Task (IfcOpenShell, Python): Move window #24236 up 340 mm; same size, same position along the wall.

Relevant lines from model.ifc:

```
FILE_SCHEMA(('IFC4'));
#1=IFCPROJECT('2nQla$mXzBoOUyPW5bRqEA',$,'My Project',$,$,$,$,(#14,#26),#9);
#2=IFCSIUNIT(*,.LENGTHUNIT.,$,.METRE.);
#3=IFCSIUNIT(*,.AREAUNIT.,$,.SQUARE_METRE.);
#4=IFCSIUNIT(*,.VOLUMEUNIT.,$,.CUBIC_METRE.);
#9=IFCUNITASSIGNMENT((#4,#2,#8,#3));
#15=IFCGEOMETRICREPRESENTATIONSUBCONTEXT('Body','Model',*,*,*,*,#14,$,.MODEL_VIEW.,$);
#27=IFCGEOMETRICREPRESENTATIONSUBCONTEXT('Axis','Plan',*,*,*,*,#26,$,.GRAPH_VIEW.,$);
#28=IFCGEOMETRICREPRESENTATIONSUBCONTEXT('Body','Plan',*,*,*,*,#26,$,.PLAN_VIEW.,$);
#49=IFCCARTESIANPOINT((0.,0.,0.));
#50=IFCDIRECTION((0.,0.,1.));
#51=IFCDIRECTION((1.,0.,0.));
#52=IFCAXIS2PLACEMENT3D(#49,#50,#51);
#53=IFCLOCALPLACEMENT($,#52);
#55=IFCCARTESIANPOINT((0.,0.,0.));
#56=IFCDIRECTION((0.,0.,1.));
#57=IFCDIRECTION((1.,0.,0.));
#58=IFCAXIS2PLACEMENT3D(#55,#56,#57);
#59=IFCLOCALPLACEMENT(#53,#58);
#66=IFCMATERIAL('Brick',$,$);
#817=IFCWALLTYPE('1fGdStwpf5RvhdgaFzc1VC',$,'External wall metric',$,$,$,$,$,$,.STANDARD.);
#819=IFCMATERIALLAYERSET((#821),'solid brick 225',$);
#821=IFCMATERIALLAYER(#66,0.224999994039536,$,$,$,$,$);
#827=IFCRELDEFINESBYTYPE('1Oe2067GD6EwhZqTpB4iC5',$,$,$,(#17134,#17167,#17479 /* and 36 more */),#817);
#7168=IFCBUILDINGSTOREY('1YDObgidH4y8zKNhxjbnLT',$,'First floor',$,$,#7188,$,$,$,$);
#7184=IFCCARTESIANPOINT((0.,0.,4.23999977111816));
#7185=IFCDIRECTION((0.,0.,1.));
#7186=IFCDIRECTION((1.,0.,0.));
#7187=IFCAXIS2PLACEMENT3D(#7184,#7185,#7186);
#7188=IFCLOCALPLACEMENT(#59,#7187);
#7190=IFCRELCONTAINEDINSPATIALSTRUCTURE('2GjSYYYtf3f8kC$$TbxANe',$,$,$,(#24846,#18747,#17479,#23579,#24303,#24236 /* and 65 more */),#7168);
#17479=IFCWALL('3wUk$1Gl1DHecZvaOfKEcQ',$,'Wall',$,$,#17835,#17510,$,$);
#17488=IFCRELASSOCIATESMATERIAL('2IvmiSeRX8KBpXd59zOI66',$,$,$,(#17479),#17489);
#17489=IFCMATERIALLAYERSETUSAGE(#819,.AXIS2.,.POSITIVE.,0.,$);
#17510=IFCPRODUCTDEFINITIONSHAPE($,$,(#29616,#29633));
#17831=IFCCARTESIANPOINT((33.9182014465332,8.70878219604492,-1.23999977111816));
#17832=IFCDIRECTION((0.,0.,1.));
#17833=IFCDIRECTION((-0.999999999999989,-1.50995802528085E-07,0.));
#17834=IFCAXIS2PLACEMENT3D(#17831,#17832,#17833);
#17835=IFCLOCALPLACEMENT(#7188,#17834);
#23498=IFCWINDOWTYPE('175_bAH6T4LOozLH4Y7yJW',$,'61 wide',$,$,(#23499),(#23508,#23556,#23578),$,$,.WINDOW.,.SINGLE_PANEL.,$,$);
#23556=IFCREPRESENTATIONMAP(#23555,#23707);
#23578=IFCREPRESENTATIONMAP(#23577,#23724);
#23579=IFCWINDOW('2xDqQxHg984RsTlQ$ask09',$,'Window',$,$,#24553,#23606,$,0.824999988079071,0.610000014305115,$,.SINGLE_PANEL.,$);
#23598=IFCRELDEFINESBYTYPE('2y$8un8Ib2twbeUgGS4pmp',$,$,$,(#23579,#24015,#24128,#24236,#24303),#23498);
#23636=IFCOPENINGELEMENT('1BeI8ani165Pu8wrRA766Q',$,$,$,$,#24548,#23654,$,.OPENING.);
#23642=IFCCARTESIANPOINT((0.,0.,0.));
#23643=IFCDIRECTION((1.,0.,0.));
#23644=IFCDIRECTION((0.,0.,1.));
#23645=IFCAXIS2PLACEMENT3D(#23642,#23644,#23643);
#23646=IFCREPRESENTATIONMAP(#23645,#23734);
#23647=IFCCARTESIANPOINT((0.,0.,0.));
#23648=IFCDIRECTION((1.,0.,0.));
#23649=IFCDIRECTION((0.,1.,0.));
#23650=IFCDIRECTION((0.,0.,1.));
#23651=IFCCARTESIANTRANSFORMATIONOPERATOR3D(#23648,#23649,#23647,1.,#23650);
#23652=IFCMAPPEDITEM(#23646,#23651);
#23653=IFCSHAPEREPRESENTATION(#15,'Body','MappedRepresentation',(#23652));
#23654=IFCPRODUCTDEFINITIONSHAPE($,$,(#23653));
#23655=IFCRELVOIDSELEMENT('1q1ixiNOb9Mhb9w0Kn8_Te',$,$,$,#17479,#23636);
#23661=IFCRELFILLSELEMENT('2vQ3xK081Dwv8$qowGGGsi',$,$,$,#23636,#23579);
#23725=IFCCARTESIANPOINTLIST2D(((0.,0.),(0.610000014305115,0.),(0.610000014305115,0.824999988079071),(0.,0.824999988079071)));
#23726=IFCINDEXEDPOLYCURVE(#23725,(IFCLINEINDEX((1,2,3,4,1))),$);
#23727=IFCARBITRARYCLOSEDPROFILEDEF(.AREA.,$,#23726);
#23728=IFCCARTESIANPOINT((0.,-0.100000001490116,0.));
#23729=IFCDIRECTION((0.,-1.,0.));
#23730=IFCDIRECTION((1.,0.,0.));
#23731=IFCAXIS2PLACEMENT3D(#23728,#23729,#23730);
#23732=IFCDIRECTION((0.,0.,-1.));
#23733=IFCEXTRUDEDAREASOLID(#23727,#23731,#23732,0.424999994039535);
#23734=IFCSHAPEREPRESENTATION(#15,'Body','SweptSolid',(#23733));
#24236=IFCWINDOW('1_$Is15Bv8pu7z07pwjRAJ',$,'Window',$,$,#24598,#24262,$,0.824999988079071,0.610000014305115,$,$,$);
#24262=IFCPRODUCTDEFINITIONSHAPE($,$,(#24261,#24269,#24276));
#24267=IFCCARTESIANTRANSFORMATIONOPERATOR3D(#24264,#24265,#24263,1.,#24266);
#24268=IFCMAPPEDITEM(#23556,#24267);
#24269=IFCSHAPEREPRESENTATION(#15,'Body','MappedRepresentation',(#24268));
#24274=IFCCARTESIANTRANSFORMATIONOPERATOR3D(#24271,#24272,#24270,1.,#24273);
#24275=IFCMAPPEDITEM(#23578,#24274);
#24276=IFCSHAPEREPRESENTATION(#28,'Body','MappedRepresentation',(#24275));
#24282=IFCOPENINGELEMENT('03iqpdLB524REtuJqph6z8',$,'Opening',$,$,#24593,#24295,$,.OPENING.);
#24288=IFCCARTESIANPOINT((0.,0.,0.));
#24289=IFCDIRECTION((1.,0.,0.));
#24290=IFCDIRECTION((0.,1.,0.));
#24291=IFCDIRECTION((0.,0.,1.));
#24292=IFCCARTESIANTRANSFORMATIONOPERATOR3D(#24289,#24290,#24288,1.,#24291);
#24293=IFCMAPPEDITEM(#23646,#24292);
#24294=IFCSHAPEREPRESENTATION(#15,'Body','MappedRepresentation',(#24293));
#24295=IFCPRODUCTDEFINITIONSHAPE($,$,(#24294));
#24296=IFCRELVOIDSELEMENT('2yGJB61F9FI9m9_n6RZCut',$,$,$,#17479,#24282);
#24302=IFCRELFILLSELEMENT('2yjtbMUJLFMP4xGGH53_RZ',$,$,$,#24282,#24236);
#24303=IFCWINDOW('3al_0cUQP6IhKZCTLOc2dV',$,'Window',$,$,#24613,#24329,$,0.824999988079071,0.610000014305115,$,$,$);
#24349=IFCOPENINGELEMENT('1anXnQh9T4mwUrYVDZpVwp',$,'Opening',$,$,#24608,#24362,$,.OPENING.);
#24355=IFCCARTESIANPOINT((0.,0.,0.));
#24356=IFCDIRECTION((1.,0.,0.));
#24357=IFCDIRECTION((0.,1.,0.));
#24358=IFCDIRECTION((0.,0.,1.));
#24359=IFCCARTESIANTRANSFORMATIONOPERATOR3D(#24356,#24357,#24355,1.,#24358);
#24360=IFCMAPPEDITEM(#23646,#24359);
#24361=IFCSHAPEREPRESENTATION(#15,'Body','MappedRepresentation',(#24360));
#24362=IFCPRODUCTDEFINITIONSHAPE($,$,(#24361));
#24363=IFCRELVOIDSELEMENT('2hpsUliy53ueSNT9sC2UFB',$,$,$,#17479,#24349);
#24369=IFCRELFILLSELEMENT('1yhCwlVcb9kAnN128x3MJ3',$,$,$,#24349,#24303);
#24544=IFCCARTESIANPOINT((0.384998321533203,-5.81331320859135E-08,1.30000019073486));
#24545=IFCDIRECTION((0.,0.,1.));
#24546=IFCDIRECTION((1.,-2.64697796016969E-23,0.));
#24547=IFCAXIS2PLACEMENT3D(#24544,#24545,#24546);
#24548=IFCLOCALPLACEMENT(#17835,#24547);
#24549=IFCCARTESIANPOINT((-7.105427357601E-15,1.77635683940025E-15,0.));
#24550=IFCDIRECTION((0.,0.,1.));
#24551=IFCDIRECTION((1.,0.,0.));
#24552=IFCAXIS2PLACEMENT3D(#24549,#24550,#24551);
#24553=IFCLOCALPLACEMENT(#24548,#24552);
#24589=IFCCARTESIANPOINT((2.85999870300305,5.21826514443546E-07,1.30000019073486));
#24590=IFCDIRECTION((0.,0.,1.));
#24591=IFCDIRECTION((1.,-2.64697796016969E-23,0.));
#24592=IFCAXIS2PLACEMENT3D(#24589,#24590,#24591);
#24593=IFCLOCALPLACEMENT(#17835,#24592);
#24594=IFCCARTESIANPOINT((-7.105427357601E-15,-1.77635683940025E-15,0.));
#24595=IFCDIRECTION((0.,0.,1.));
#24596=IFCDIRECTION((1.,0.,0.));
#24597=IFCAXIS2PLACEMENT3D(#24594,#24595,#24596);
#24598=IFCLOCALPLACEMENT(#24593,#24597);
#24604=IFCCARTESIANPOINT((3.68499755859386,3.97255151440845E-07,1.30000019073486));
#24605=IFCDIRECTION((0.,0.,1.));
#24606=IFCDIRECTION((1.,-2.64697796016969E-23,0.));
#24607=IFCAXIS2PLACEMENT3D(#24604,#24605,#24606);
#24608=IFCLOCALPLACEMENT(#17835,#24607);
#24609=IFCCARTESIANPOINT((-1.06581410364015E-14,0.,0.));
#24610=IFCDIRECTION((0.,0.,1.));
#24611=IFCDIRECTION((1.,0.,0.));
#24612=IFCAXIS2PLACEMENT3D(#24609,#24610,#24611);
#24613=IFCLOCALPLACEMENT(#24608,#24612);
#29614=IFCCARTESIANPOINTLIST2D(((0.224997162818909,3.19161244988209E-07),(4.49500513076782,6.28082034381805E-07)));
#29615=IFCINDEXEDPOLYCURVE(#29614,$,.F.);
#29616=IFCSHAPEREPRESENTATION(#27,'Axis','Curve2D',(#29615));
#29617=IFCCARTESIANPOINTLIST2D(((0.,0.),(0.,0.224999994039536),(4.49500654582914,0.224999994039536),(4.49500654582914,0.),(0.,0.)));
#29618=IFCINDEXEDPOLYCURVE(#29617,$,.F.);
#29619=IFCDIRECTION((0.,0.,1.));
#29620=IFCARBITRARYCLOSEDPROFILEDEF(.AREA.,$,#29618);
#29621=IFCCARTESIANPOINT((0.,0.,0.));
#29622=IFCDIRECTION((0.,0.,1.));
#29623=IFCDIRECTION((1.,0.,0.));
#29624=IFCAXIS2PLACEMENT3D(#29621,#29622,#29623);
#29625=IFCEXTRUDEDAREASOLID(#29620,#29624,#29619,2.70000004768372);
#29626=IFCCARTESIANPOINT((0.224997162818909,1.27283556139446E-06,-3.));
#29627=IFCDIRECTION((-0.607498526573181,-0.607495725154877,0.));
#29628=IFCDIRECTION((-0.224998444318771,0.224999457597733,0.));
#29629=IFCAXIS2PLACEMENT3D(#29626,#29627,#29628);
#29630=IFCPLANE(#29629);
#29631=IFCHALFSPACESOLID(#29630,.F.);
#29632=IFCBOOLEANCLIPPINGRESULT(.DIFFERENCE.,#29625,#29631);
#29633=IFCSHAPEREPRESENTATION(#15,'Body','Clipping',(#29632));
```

```python
import numpy as np
import ifcopenshell
import ifcopenshell.api.geometry
import ifcopenshell.util.placement
import ifcopenshell.util.unit

model = ifcopenshell.open("model.ifc")
unit_scale = ifcopenshell.util.unit.calculate_unit_scale(model)

window = model.by_guid("1_$Is15Bv8pu7z07pwjRAJ")
opening = window.FillsVoids[0].RelatingOpeningElement
dz = 0.34

shift = np.array([0.0, 0.0, dz])
# The window is placed relative to its opening, so it follows when the opening moves.
matrix = ifcopenshell.util.placement.get_local_placement(opening.ObjectPlacement)
matrix[:3, 3] += shift
ifcopenshell.api.geometry.edit_object_placement(
    model, product=opening, matrix=matrix, is_si=False, should_transform_children=True
)

print(f"moved by {dz * unit_scale:+.3f} m")

model.write("model-out.ifc")
```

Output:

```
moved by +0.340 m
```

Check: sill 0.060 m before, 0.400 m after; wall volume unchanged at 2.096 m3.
